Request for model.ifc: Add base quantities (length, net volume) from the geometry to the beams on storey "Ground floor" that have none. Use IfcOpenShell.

First a look at what the model holds.

```python
import ifcopenshell
import ifcopenshell.util.element
import ifcopenshell.util.unit

model = ifcopenshell.open("model.ifc")
print(model.schema)
for unit_type in ("LENGTHUNIT", "AREAUNIT", "VOLUMEUNIT"):
    print(unit_type, ifcopenshell.util.unit.calculate_unit_scale(model, unit_type))
storey = next(s for s in model.by_type("IfcBuildingStorey") if s.Name == "Ground floor")
beams = [e for e in ifcopenshell.util.element.get_decomposition(storey) if e.is_a("IfcBeam")]
for e in sorted(beams, key=lambda e: e.id()):
    print(e.id(), e.is_a(), e.Name, list(ifcopenshell.util.element.get_psets(e, qtos_only=True)), sep=" | ")
```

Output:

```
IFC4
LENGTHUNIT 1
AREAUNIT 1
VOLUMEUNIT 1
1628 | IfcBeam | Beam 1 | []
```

```python
import ifcopenshell
import ifcopenshell.api.pset
import ifcopenshell.geom
import ifcopenshell.util.element
import ifcopenshell.util.shape
import ifcopenshell.util.unit

model = ifcopenshell.open("model.ifc")
unit_scale = ifcopenshell.util.unit.calculate_unit_scale(model)
volume_scale = ifcopenshell.util.unit.calculate_unit_scale(model, "VOLUMEUNIT")
settings = ifcopenshell.geom.settings()

storey = next(s for s in model.by_type("IfcBuildingStorey") if s.Name == "Ground floor")
beams = [e for e in ifcopenshell.util.element.get_decomposition(storey) if e.is_a("IfcBeam")]

for e in sorted(beams, key=lambda e: e.id()):
    if ifcopenshell.util.element.get_psets(e, qtos_only=True, should_inherit=False):
        continue
    # Geometry comes back in metres, in the element's own axes.
    shape = ifcopenshell.geom.create_shape(settings, e)
    values = {
        "Length": ifcopenshell.util.shape.get_max_xyz(shape.geometry) / unit_scale,
        "NetVolume": ifcopenshell.util.shape.get_volume(shape.geometry) / volume_scale,
    }
    qto = ifcopenshell.api.pset.add_qto(model, product=e, name="Qto_BeamBaseQuantities")
    ifcopenshell.api.pset.edit_qto(model, qto=qto, properties=values)
    print(e.id(), {k: round(v, 3) for k, v in values.items()})

model.write("model_edited.ifc")
```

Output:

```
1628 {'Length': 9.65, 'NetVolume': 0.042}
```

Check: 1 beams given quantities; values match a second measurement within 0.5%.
